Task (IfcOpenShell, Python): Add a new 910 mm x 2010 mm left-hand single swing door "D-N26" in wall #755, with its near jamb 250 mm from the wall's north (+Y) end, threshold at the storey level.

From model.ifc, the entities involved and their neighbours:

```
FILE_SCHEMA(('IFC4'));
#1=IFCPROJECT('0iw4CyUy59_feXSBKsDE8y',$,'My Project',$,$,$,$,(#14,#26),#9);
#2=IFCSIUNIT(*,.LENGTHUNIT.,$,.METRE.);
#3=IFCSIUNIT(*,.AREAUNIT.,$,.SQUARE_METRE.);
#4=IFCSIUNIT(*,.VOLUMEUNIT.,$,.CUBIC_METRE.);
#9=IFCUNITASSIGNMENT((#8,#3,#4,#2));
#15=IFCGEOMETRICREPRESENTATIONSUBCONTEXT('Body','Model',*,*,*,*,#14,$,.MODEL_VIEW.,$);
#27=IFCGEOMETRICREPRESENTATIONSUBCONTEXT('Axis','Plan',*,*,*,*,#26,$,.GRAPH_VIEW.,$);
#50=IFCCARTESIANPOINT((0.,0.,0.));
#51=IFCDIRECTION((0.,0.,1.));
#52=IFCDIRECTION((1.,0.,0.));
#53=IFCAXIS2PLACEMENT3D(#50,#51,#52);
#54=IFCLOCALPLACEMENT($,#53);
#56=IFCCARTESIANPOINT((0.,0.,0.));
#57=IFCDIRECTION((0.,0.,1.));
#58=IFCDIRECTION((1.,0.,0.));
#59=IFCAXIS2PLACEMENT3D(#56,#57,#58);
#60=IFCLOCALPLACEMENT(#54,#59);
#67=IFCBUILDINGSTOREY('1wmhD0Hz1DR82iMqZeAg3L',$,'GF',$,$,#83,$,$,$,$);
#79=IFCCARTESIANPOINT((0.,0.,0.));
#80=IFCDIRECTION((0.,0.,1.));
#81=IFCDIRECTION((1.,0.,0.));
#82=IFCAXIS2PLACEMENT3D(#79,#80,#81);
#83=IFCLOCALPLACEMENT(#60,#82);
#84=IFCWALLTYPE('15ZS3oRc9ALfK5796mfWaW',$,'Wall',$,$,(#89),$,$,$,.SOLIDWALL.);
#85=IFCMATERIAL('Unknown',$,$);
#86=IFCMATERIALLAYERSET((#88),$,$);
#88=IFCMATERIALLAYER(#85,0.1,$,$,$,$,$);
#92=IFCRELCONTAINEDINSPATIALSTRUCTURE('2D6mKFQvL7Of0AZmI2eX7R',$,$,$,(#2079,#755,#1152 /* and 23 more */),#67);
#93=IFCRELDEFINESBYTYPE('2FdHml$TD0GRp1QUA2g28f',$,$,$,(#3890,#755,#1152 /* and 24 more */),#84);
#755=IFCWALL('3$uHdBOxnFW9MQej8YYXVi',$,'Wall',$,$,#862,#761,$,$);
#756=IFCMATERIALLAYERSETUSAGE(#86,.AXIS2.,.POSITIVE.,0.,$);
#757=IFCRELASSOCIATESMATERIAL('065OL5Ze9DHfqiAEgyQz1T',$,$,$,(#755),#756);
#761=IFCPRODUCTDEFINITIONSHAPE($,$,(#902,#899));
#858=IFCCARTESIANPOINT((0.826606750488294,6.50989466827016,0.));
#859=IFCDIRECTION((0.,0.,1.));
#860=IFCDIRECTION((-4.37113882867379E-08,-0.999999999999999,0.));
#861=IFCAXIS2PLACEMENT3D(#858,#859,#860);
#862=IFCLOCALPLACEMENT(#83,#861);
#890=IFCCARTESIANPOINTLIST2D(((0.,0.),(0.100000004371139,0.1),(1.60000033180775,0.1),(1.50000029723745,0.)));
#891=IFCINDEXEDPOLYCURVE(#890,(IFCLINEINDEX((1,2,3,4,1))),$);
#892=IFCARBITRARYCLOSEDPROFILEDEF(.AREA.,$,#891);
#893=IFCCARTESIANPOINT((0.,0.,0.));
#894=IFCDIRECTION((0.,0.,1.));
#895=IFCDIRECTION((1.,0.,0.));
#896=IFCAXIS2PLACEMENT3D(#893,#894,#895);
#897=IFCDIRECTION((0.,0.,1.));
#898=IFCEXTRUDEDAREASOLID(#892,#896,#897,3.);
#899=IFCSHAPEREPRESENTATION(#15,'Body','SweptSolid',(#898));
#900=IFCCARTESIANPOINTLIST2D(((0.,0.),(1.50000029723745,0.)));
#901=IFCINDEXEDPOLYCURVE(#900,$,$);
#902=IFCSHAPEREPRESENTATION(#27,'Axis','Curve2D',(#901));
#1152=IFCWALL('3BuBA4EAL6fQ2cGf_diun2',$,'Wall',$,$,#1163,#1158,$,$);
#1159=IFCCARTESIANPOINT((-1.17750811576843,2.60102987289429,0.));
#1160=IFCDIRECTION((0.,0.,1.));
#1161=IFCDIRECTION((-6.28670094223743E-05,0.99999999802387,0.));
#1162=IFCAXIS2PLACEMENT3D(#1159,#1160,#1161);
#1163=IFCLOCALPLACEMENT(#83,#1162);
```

```python
import numpy as np
import ifcopenshell
import ifcopenshell.api.feature
import ifcopenshell.api.geometry
import ifcopenshell.api.root
import ifcopenshell.api.spatial
import ifcopenshell.geom
import ifcopenshell.util.element
import ifcopenshell.util.placement
import ifcopenshell.util.representation
import ifcopenshell.util.shape
import ifcopenshell.util.unit

model = ifcopenshell.open("model.ifc")
unit_scale = ifcopenshell.util.unit.calculate_unit_scale(model)
settings = ifcopenshell.geom.settings()


def volume(element):
    """Net volume in cubic metres, openings subtracted."""
    shape = ifcopenshell.geom.create_shape(settings, element)
    return ifcopenshell.util.shape.get_volume(shape.geometry)


wall = model.by_guid("3$uHdBOxnFW9MQej8YYXVi")
storey = ifcopenshell.util.element.get_container(wall, ifc_class="IfcBuildingStorey")
context = ifcopenshell.util.representation.get_context(model, "Model", "Body", "MODEL_VIEW")
before = volume(wall)

width, height, from_end, sill = 0.91, 2.01, 0.25, 0.0  # metres

# The wall runs along its own X axis, and the end named is its -X end.
wall_shape = ifcopenshell.geom.create_shape(settings, wall)
x, y, z = ifcopenshell.util.shape.get_vertices(wall_shape.geometry).T
start = x.min() + from_end
face, thickness = float(y.min()), float(y.max() - y.min())
wall_matrix = ifcopenshell.util.placement.get_local_placement(wall.ObjectPlacement)
level = ifcopenshell.util.placement.get_local_placement(storey.ObjectPlacement)[2, 3]


def in_wall(x, y):
    """Placement at x, y metres in the wall's axes, at sill height."""
    matrix = wall_matrix.copy()
    matrix[:, 3] = wall_matrix @ np.array([x / unit_scale, y / unit_scale, 0.0, 1.0])
    matrix[2, 3] = level + sill / unit_scale
    return matrix


# Opening: a box that overshoots both wall faces by 50 mm.
opening = ifcopenshell.api.root.create_entity(model, ifc_class="IfcOpeningElement", predefined_type="OPENING")
box = ifcopenshell.api.geometry.add_wall_representation(
    model, context=context, length=width, height=height, thickness=thickness + 0.1
)
ifcopenshell.api.geometry.assign_representation(model, product=opening, representation=box)
ifcopenshell.api.geometry.edit_object_placement(model, product=opening, matrix=in_wall(start, face - 0.05), is_si=False)
ifcopenshell.api.feature.add_feature(model, feature=opening, element=wall)

door = ifcopenshell.api.root.create_entity(model, ifc_class="IfcDoor", name="D-N26", predefined_type="DOOR")
door.OverallWidth, door.OverallHeight = width / unit_scale, height / unit_scale
door.OperationType = "SINGLE_SWING_LEFT"
body = ifcopenshell.api.geometry.add_door_representation(
    model,
    context=context,
    overall_width=door.OverallWidth,
    overall_height=door.OverallHeight,
    operation_type="SINGLE_SWING_LEFT",
    lining_properties={"LiningDepth": thickness / unit_scale, "ThresholdDepth": thickness / unit_scale},
)
ifcopenshell.api.geometry.assign_representation(model, product=door, representation=body)
ifcopenshell.api.spatial.assign_container(model, products=[door], relating_structure=storey)
ifcopenshell.api.feature.add_filling(model, opening=opening, element=door)

# The lining spans the wall, so the door starts at the wall face.
ifcopenshell.api.geometry.edit_object_placement(model, product=door, matrix=in_wall(start, face), is_si=False)

after = volume(wall)

print(f"wall volume {before:.3f} -> {after:.3f} m3")

model.write("model_rev.ifc")
```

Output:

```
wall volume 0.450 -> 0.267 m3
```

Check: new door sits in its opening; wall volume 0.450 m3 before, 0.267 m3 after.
